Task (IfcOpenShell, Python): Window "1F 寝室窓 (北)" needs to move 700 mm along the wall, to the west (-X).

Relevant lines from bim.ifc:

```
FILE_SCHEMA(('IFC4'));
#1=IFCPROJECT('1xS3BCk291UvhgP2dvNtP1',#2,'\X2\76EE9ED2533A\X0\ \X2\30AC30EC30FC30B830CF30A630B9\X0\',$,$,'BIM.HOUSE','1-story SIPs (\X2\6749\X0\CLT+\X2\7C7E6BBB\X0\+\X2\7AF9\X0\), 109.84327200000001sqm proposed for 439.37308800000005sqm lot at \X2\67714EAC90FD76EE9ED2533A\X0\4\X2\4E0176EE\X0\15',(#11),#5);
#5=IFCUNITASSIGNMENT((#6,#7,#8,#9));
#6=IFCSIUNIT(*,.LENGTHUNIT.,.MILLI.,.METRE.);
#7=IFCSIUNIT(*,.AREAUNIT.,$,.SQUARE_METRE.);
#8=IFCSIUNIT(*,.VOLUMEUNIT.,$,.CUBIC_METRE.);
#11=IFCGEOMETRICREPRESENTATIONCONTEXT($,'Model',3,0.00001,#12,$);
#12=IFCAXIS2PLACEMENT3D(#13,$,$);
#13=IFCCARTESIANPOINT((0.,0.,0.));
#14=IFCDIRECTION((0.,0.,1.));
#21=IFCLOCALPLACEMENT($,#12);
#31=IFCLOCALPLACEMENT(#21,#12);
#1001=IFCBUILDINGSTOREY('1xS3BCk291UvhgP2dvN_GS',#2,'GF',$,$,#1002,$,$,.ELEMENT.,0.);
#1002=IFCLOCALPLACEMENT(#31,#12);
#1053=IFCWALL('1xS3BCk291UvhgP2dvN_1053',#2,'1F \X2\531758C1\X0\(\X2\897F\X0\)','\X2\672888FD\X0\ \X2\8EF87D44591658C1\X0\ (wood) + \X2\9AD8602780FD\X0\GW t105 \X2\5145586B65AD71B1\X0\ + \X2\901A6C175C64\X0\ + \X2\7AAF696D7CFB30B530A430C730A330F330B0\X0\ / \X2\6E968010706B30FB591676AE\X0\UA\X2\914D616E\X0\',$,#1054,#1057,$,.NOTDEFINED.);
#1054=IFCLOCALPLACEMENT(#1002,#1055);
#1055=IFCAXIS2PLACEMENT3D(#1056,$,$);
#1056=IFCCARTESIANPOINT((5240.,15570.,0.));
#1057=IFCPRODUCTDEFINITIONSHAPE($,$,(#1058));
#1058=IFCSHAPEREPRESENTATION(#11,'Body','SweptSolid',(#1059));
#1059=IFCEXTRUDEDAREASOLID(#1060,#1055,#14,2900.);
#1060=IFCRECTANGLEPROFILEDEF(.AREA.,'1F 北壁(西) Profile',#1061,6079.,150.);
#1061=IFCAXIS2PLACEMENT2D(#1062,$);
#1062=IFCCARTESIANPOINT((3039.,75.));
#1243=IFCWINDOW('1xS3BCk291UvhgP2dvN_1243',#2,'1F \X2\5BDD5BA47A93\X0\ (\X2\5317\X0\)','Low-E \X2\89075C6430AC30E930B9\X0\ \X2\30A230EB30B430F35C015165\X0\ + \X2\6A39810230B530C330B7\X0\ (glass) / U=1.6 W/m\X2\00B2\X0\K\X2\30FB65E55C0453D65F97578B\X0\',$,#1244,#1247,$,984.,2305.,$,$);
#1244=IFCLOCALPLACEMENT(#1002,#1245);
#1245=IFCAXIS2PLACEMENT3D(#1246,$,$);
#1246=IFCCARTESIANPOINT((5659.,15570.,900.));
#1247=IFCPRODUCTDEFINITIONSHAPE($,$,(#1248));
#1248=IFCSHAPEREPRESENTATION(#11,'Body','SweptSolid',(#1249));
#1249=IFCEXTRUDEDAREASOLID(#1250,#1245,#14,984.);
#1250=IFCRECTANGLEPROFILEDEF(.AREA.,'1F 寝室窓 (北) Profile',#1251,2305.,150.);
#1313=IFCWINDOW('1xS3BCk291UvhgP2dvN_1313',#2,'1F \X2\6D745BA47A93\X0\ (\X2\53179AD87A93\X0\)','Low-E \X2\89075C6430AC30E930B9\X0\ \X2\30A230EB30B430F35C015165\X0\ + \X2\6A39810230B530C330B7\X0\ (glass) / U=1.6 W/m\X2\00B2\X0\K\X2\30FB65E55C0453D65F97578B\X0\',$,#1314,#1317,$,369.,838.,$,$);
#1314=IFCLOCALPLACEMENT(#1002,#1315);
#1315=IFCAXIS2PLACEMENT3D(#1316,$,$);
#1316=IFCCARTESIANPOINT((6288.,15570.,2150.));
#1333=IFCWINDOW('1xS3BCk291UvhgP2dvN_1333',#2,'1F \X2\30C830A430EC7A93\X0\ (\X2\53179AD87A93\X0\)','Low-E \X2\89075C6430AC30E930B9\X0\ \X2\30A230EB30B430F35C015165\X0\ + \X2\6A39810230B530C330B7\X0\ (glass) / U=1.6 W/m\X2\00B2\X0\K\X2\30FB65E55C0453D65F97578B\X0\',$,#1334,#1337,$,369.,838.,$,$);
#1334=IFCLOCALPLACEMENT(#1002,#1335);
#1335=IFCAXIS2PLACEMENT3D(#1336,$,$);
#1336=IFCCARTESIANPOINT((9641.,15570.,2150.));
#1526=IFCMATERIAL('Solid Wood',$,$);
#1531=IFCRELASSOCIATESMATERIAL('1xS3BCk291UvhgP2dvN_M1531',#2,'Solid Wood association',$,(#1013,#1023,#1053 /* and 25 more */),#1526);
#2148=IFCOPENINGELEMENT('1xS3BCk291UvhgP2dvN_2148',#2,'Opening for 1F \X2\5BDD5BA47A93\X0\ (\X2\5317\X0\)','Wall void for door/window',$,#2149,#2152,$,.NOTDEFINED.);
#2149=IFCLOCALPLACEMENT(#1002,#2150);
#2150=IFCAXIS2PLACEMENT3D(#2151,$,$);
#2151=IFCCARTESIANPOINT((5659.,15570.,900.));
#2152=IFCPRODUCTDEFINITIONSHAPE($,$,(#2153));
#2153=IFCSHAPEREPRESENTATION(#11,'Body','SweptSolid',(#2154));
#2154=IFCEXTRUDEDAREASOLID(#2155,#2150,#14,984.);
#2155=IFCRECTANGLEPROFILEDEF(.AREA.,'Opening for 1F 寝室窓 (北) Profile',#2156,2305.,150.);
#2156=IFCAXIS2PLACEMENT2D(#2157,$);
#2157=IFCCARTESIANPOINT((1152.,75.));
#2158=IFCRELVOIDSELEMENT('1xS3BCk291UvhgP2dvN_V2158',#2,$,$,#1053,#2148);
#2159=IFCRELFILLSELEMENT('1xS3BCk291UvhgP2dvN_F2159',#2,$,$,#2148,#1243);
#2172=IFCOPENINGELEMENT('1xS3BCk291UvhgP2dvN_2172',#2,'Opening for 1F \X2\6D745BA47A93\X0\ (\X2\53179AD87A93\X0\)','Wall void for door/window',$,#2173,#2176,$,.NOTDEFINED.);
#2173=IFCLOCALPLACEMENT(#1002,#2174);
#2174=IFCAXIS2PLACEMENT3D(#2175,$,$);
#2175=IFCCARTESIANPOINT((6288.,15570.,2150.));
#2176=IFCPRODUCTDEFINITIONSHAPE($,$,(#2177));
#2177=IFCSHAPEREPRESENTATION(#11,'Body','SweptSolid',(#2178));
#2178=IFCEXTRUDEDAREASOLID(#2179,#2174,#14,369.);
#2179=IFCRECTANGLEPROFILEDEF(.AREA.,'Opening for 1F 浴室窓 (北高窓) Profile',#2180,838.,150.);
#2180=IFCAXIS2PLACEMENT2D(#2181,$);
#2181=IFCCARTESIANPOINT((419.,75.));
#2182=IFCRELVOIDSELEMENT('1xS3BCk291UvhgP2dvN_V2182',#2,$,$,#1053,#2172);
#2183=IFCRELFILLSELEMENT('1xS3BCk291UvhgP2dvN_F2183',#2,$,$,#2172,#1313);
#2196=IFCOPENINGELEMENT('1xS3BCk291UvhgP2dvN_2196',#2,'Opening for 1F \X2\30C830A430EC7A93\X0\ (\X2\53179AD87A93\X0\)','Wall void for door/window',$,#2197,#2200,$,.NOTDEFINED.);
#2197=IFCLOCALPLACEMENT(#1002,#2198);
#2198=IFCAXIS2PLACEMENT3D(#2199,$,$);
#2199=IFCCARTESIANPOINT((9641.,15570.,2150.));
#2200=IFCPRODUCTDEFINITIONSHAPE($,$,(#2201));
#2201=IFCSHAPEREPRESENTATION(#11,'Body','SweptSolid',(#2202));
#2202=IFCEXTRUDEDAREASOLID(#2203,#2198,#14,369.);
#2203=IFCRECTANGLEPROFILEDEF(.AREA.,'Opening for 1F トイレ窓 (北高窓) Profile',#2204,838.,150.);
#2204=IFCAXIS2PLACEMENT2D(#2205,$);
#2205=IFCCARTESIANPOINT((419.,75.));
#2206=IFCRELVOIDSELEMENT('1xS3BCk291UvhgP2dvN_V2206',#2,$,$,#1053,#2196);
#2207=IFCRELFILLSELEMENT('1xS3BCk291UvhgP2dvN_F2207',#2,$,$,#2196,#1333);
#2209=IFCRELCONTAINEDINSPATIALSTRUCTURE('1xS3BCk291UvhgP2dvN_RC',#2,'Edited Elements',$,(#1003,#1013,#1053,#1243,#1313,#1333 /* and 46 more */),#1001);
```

```python
import ifcopenshell
import ifcopenshell.api.geometry
import ifcopenshell.util.placement
import ifcopenshell.util.unit

model = ifcopenshell.open("bim.ifc")
unit_scale = ifcopenshell.util.unit.calculate_unit_scale(model)

window = model.by_guid("1xS3BCk291UvhgP2dvN_1243")
opening = window.FillsVoids[0].RelatingOpeningElement
wall = opening.VoidsElements[0].RelatingBuildingElement

wall_matrix = ifcopenshell.util.placement.get_local_placement(wall.ObjectPlacement)
shift = wall_matrix[:3, 0] * -0.7 / unit_scale
before = ifcopenshell.util.placement.get_local_placement(window.ObjectPlacement)[:3, 3].copy()

# The window is not placed relative to its opening, so move both.
for product in (opening, window):
    matrix = ifcopenshell.util.placement.get_local_placement(product.ObjectPlacement)
    matrix[:3, 3] += shift
    ifcopenshell.api.geometry.edit_object_placement(model, product=product, matrix=matrix, is_si=False)

after = ifcopenshell.util.placement.get_local_placement(window.ObjectPlacement)[:3, 3]
print("window moved by", (after - before).round(3) + 0.0)

model.write("bim-out.ifc")
```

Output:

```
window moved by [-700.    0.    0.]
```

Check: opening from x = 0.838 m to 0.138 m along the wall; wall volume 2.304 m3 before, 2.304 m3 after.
